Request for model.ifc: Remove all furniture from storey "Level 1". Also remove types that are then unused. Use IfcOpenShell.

First a look at what the model holds.

```python
import ifcopenshell
import ifcopenshell.util.element

model = ifcopenshell.open("model.ifc")
print(model.schema)
storey = next(s for s in model.by_type("IfcBuildingStorey") if s.Name == "Level 1")
furniture = [e for e in ifcopenshell.util.element.get_decomposition(storey) if e.is_a("IfcFurnishingElement")]
seen = {}
for e in furniture:
    element_type = ifcopenshell.util.element.get_type(e)
    name = element_type.Name if element_type not in (None, e) else None
    seen[name] = seen.get(name, 0) + 1
for name, count in sorted(seen.items(), key=str):
    print(count, "x", name)
```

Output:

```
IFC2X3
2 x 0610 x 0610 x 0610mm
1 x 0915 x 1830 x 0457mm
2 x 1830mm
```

```python
import ifcopenshell
import ifcopenshell.api.root
import ifcopenshell.util.element

model = ifcopenshell.open("model.ifc")

storey = next(s for s in model.by_type("IfcBuildingStorey") if s.Name == "Level 1")
furniture = [e for e in ifcopenshell.util.element.get_decomposition(storey) if e.is_a("IfcFurnishingElement")]
types = {ifcopenshell.util.element.get_type(e) for e in furniture} - {None, *furniture}

for e in furniture:
    ifcopenshell.api.root.remove_product(model, product=e)
print(len(furniture), "removed")

unused = [t for t in types if not ifcopenshell.util.element.get_types(t)]
for t in unused:
    ifcopenshell.api.root.remove_product(model, product=t)
print(len(unused), "unused types removed")

model.write("model_rev.ifc")
```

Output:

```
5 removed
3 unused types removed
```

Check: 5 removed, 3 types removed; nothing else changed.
